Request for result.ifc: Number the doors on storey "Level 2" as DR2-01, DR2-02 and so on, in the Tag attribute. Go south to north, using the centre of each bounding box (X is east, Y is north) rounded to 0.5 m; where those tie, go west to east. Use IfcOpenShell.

First a look at what the model holds.

```python
import ifcopenshell
import ifcopenshell.util.element
import ifcopenshell.util.placement

model = ifcopenshell.open("result.ifc")
print(model.schema)
storey = next(s for s in model.by_type("IfcBuildingStorey") if s.Name == "Level 2")
doors = [e for e in ifcopenshell.util.element.get_decomposition(storey) if e.is_a("IfcDoor")]
for e in sorted(doors, key=lambda e: e.id()):
    origin = ifcopenshell.util.placement.get_local_placement(e.ObjectPlacement)[:3, 3]
    print(e.id(), e.Tag, e.Name, origin.round(2) + 0.0, sep=" | ")
```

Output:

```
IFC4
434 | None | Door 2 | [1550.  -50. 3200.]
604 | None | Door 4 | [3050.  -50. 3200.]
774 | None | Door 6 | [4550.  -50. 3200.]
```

```python
import ifcopenshell
import ifcopenshell.geom
import ifcopenshell.util.element
import ifcopenshell.util.shape

model = ifcopenshell.open("result.ifc")
settings = ifcopenshell.geom.settings()
settings.set("use-world-coords", True)


def centre(element):
    shape = ifcopenshell.geom.create_shape(settings, element)
    return ifcopenshell.util.shape.get_bbox_centroid(shape.geometry)


storey = next(s for s in model.by_type("IfcBuildingStorey") if s.Name == "Level 2")
doors = [e for e in ifcopenshell.util.element.get_decomposition(storey) if e.is_a("IfcDoor")]

# Insertion points can sit at a corner or the storey origin, so sort by the geometry (in metres).
centres = {e: centre(e) for e in doors}
doors.sort(key=lambda e: (round(centres[e][1] / 0.5), centres[e][0]))

for i, e in enumerate(doors, start=1):
    number = f"DR2-{i:02d}"
    e.Tag = number
    print(e.id(), number)

model.write("result_rev.ifc")
```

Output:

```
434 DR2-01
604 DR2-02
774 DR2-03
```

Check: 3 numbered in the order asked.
